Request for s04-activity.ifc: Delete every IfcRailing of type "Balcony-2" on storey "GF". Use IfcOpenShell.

First a look at what the model holds.

```python
import ifcopenshell
import ifcopenshell.util.element

model = ifcopenshell.open("s04-activity.ifc")
print(model.schema)
storey = next(s for s in model.by_type("IfcBuildingStorey") if s.Name == "GF")
railings = [e for e in ifcopenshell.util.element.get_decomposition(storey) if e.is_a("IfcRailing")]
seen = {}
for e in railings:
    element_type = ifcopenshell.util.element.get_type(e)
    name = element_type.Name if element_type not in (None, e) else None
    seen[name] = seen.get(name, 0) + 1
for name, count in sorted(seen.items(), key=str):
    print(count, "x", name)
```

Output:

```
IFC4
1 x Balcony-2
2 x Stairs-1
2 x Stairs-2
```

```python
import ifcopenshell
import ifcopenshell.api.root
import ifcopenshell.util.element

model = ifcopenshell.open("s04-activity.ifc")

storey = next(s for s in model.by_type("IfcBuildingStorey") if s.Name == "GF")
railings = [e for e in ifcopenshell.util.element.get_decomposition(storey) if e.is_a("IfcRailing")]
targets = [e for e in railings if (t := ifcopenshell.util.element.get_type(e)) not in (None, e) and t.Name == "Balcony-2"]

for e in targets:
    ifcopenshell.api.root.remove_product(model, product=e)
print(len(targets), "removed")

model.write("s04-activity_rev.ifc")
```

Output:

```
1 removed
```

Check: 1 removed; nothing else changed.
